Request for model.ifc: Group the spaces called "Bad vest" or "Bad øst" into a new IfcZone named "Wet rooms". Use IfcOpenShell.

First a look at what the model holds.

```python
import ifcopenshell

model = ifcopenshell.open("model.ifc")
print(model.schema)
seen = {}
for space in model.by_type("IfcSpace"):
    seen[space.LongName] = seen.get(space.LongName, 0) + 1
for name, count in sorted(seen.items(), key=str):
    print(count, "x", name)
print("zones:", [z.Name for z in model.by_type("IfcZone")][:20])
```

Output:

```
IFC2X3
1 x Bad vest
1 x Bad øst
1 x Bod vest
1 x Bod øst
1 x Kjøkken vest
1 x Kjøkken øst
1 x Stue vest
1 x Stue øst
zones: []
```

```python
import ifcopenshell
import ifcopenshell.api.group
import ifcopenshell.api.root

model = ifcopenshell.open("model.ifc")

names = {"Bad vest", "Bad øst"}
spaces = [s for s in model.by_type("IfcSpace") if s.LongName in names]

zone = ifcopenshell.api.root.create_entity(model, ifc_class="IfcZone", name="Wet rooms")
ifcopenshell.api.group.assign_group(model, products=spaces, group=zone)
print(len(spaces), "spaces in", zone.Name)

model.write("model_rev.ifc")
```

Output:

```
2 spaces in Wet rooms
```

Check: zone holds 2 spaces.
